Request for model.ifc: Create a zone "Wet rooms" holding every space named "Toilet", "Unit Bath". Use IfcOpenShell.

First a look at what the model holds.

```python
import ifcopenshell

model = ifcopenshell.open("model.ifc")
print(model.schema)
seen = {}
for space in model.by_type("IfcSpace"):
    seen[space.LongName] = seen.get(space.LongName, 0) + 1
for name, count in sorted(seen.items(), key=str):
    print(count, "x", name)
print("zones:", [z.Name for z in model.by_type("IfcZone")][:20])
```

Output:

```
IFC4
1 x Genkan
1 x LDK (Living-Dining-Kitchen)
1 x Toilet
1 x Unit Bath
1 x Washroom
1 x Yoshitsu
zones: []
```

```python
import ifcopenshell
import ifcopenshell.api.group
import ifcopenshell.api.root

model = ifcopenshell.open("model.ifc")

names = {"Toilet", "Unit Bath"}
spaces = [s for s in model.by_type("IfcSpace") if s.LongName in names]

zone = ifcopenshell.api.root.create_entity(model, ifc_class="IfcZone", name="Wet rooms")
ifcopenshell.api.group.assign_group(model, products=spaces, group=zone)
print(len(spaces), "spaces in", zone.Name)

model.write("model_v2.ifc")
```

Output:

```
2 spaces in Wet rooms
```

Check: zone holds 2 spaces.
